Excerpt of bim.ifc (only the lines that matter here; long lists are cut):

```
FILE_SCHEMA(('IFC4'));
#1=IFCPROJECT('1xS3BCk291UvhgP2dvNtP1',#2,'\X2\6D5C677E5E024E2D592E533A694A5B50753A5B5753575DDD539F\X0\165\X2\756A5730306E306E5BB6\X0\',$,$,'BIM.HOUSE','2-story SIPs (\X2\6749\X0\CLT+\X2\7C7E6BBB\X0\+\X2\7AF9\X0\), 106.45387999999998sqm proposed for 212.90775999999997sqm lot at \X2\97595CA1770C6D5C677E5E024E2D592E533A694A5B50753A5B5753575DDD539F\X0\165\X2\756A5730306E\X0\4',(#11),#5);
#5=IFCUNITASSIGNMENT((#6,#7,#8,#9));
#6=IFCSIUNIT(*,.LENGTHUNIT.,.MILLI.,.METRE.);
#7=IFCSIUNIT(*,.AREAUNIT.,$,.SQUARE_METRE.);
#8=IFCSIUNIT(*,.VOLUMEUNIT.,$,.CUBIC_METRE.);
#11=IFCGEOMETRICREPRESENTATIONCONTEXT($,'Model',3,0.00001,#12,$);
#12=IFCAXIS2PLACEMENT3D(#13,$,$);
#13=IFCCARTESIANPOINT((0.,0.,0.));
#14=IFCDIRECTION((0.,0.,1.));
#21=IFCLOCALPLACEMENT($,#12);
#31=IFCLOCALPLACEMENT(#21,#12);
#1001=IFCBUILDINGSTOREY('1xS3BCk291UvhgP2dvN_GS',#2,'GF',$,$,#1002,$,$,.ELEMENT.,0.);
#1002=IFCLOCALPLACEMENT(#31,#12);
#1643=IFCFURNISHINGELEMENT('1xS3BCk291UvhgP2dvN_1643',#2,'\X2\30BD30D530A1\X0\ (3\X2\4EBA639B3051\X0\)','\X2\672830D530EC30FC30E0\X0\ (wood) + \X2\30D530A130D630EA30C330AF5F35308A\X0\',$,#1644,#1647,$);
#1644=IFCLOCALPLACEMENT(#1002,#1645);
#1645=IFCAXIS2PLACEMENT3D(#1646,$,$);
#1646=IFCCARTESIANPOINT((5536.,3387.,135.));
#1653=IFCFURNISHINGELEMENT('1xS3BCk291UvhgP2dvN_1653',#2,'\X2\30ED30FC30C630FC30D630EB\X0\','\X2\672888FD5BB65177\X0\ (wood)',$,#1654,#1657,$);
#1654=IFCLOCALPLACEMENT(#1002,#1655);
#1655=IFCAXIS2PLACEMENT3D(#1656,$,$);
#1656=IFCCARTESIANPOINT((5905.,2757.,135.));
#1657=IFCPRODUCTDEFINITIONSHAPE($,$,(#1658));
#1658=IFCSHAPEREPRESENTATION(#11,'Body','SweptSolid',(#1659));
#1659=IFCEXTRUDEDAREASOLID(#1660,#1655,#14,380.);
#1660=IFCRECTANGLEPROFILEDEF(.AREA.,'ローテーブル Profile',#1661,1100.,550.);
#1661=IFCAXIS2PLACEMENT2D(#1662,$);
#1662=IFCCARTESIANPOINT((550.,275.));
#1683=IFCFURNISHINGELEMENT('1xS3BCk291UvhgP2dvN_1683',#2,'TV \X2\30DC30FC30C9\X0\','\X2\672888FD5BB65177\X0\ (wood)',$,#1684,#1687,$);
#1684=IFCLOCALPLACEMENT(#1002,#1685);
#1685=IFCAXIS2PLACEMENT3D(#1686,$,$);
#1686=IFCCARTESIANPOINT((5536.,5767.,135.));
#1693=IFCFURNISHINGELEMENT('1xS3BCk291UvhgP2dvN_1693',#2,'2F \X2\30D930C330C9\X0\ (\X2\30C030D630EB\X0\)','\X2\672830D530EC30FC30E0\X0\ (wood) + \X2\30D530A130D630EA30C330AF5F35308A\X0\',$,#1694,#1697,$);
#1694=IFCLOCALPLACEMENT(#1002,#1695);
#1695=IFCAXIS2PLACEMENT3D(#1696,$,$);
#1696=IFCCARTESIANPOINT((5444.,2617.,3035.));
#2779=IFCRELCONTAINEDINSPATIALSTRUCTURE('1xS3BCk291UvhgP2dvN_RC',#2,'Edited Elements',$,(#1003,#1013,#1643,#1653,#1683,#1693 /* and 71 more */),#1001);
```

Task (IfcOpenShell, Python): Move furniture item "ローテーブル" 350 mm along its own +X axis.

```python
import ifcopenshell
import ifcopenshell.api.geometry
import ifcopenshell.util.placement
import ifcopenshell.util.unit

model = ifcopenshell.open("bim.ifc")
unit_scale = ifcopenshell.util.unit.calculate_unit_scale(model)

item = model.by_guid("1xS3BCk291UvhgP2dvN_1653")
matrix = ifcopenshell.util.placement.get_local_placement(item.ObjectPlacement)
matrix[:3, 3] += matrix[:3, 0] * 0.35 / unit_scale
ifcopenshell.api.geometry.edit_object_placement(model, product=item, matrix=matrix, is_si=False)

print(ifcopenshell.util.placement.get_local_placement(item.ObjectPlacement).round(3) + 0.0)

model.write("bim_rev.ifc")
```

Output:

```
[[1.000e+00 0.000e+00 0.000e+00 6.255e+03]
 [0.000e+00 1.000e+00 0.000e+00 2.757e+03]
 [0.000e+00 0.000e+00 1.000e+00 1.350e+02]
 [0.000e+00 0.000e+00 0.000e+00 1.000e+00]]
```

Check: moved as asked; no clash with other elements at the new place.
